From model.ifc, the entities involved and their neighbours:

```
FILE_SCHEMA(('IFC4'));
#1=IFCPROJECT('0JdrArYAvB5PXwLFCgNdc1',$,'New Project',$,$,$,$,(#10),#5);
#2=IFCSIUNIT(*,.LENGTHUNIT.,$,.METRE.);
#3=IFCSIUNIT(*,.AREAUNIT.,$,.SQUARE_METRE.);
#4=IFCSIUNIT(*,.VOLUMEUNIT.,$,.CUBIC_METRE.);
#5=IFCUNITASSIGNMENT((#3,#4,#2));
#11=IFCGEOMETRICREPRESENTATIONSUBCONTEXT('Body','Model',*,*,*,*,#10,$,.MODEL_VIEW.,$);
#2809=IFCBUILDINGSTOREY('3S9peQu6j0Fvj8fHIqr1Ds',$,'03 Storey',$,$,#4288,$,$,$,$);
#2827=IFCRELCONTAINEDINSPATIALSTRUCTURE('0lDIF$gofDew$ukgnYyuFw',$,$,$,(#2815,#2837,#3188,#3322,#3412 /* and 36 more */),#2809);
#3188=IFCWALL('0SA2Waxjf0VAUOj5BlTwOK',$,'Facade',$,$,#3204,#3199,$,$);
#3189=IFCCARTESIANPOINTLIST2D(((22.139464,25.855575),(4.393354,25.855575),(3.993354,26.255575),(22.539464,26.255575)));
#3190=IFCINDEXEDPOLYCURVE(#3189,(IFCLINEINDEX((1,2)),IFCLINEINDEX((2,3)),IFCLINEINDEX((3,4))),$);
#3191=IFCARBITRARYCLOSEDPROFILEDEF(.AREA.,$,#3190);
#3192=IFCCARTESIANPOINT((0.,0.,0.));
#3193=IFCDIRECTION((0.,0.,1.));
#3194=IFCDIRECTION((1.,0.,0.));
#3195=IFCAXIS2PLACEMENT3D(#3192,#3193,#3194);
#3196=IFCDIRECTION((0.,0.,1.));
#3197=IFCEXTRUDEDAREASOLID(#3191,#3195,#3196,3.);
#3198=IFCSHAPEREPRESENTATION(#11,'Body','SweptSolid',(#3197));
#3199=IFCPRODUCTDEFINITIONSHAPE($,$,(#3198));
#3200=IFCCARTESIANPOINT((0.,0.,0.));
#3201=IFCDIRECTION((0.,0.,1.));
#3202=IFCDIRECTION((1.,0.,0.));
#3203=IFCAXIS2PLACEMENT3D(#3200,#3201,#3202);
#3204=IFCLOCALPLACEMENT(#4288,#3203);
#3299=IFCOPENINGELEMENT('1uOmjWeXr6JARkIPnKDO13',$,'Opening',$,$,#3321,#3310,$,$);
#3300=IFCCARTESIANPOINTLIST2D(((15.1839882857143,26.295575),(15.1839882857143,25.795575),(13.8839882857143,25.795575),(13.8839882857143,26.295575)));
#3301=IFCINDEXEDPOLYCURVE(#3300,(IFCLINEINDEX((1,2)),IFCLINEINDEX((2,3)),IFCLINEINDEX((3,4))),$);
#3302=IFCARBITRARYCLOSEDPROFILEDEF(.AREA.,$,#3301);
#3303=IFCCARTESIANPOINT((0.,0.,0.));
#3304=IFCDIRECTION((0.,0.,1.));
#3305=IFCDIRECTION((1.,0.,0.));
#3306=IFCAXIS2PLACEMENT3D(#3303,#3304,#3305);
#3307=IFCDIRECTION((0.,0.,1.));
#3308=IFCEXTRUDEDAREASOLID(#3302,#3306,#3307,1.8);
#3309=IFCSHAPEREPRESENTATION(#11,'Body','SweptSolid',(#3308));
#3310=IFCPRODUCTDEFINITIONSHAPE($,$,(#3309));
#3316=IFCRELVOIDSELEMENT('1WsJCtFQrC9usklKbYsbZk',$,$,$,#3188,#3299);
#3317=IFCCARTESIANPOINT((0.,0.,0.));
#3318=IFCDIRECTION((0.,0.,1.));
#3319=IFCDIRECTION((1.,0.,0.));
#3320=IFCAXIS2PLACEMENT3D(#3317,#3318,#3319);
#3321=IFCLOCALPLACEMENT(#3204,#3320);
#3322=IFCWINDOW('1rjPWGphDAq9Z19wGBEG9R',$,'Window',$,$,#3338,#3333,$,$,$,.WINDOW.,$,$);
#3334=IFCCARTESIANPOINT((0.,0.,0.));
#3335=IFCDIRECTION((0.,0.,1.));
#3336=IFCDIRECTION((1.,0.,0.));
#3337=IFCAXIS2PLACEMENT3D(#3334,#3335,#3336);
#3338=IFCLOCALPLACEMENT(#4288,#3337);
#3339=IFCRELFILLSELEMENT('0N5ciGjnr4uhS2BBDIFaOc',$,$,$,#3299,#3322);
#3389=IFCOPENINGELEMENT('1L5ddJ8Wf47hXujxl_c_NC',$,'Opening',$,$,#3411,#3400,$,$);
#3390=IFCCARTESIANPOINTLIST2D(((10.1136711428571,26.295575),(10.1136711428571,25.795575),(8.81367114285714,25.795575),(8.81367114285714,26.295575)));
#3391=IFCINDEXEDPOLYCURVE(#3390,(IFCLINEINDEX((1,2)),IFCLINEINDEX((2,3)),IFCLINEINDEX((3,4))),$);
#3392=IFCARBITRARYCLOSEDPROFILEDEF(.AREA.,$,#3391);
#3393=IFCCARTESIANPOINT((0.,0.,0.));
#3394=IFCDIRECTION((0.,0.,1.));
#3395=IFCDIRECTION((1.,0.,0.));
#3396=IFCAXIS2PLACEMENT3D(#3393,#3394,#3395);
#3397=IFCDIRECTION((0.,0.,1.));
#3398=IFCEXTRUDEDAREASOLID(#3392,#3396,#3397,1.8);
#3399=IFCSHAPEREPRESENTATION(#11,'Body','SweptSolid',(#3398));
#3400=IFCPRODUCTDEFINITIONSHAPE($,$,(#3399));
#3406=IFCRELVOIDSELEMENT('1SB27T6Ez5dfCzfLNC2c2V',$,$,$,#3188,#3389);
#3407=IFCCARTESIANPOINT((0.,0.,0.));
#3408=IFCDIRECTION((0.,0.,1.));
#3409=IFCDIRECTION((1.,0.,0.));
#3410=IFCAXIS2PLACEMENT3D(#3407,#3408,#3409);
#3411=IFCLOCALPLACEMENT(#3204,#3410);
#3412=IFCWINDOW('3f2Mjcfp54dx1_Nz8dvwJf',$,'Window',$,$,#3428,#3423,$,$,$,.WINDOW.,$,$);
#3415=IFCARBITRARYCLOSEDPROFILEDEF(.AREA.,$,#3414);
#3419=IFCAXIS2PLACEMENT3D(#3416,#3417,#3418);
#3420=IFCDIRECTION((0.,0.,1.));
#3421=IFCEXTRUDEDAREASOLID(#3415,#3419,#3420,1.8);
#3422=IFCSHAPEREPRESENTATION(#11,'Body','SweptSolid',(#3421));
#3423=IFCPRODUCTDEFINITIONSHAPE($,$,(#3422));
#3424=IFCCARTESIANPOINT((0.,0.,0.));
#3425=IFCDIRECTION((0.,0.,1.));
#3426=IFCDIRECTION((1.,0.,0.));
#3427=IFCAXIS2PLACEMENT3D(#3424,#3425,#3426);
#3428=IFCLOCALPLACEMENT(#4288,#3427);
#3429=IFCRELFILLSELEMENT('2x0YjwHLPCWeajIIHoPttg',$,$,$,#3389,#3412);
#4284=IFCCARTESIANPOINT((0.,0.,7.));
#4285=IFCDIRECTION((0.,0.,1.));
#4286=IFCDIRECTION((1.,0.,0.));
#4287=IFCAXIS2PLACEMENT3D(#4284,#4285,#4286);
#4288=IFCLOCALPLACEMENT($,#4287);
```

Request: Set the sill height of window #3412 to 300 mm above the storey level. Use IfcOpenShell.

```python
import numpy as np
import ifcopenshell
import ifcopenshell.api.geometry
import ifcopenshell.geom
import ifcopenshell.util.element
import ifcopenshell.util.placement
import ifcopenshell.util.shape
import ifcopenshell.util.unit

model = ifcopenshell.open("model.ifc")
unit_scale = ifcopenshell.util.unit.calculate_unit_scale(model)

window = model.by_guid("3f2Mjcfp54dx1_Nz8dvwJf")
opening = window.FillsVoids[0].RelatingOpeningElement
storey = ifcopenshell.util.element.get_container(window, ifc_class="IfcBuildingStorey")
level = ifcopenshell.util.placement.get_local_placement(storey.ObjectPlacement)[2, 3]

# The opening's origin need not be at the sill, so measure its lowest point.
shape = ifcopenshell.geom.create_shape(ifcopenshell.geom.settings(), opening)
bottom = ifcopenshell.util.shape.get_shape_bottom_elevation(shape, shape.geometry) / unit_scale
dz = level + 0.3 / unit_scale - bottom

shift = np.array([0.0, 0.0, dz])
# The window is not placed relative to its opening, so move both.
for product in (opening, window):
    matrix = ifcopenshell.util.placement.get_local_placement(product.ObjectPlacement)
    matrix[:3, 3] += shift
    ifcopenshell.api.geometry.edit_object_placement(model, product=product, matrix=matrix, is_si=False)

print(f"moved by {dz * unit_scale:+.3f} m")

model.write("model_v2.ifc")
```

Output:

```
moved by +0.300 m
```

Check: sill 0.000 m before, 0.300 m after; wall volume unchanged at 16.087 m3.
